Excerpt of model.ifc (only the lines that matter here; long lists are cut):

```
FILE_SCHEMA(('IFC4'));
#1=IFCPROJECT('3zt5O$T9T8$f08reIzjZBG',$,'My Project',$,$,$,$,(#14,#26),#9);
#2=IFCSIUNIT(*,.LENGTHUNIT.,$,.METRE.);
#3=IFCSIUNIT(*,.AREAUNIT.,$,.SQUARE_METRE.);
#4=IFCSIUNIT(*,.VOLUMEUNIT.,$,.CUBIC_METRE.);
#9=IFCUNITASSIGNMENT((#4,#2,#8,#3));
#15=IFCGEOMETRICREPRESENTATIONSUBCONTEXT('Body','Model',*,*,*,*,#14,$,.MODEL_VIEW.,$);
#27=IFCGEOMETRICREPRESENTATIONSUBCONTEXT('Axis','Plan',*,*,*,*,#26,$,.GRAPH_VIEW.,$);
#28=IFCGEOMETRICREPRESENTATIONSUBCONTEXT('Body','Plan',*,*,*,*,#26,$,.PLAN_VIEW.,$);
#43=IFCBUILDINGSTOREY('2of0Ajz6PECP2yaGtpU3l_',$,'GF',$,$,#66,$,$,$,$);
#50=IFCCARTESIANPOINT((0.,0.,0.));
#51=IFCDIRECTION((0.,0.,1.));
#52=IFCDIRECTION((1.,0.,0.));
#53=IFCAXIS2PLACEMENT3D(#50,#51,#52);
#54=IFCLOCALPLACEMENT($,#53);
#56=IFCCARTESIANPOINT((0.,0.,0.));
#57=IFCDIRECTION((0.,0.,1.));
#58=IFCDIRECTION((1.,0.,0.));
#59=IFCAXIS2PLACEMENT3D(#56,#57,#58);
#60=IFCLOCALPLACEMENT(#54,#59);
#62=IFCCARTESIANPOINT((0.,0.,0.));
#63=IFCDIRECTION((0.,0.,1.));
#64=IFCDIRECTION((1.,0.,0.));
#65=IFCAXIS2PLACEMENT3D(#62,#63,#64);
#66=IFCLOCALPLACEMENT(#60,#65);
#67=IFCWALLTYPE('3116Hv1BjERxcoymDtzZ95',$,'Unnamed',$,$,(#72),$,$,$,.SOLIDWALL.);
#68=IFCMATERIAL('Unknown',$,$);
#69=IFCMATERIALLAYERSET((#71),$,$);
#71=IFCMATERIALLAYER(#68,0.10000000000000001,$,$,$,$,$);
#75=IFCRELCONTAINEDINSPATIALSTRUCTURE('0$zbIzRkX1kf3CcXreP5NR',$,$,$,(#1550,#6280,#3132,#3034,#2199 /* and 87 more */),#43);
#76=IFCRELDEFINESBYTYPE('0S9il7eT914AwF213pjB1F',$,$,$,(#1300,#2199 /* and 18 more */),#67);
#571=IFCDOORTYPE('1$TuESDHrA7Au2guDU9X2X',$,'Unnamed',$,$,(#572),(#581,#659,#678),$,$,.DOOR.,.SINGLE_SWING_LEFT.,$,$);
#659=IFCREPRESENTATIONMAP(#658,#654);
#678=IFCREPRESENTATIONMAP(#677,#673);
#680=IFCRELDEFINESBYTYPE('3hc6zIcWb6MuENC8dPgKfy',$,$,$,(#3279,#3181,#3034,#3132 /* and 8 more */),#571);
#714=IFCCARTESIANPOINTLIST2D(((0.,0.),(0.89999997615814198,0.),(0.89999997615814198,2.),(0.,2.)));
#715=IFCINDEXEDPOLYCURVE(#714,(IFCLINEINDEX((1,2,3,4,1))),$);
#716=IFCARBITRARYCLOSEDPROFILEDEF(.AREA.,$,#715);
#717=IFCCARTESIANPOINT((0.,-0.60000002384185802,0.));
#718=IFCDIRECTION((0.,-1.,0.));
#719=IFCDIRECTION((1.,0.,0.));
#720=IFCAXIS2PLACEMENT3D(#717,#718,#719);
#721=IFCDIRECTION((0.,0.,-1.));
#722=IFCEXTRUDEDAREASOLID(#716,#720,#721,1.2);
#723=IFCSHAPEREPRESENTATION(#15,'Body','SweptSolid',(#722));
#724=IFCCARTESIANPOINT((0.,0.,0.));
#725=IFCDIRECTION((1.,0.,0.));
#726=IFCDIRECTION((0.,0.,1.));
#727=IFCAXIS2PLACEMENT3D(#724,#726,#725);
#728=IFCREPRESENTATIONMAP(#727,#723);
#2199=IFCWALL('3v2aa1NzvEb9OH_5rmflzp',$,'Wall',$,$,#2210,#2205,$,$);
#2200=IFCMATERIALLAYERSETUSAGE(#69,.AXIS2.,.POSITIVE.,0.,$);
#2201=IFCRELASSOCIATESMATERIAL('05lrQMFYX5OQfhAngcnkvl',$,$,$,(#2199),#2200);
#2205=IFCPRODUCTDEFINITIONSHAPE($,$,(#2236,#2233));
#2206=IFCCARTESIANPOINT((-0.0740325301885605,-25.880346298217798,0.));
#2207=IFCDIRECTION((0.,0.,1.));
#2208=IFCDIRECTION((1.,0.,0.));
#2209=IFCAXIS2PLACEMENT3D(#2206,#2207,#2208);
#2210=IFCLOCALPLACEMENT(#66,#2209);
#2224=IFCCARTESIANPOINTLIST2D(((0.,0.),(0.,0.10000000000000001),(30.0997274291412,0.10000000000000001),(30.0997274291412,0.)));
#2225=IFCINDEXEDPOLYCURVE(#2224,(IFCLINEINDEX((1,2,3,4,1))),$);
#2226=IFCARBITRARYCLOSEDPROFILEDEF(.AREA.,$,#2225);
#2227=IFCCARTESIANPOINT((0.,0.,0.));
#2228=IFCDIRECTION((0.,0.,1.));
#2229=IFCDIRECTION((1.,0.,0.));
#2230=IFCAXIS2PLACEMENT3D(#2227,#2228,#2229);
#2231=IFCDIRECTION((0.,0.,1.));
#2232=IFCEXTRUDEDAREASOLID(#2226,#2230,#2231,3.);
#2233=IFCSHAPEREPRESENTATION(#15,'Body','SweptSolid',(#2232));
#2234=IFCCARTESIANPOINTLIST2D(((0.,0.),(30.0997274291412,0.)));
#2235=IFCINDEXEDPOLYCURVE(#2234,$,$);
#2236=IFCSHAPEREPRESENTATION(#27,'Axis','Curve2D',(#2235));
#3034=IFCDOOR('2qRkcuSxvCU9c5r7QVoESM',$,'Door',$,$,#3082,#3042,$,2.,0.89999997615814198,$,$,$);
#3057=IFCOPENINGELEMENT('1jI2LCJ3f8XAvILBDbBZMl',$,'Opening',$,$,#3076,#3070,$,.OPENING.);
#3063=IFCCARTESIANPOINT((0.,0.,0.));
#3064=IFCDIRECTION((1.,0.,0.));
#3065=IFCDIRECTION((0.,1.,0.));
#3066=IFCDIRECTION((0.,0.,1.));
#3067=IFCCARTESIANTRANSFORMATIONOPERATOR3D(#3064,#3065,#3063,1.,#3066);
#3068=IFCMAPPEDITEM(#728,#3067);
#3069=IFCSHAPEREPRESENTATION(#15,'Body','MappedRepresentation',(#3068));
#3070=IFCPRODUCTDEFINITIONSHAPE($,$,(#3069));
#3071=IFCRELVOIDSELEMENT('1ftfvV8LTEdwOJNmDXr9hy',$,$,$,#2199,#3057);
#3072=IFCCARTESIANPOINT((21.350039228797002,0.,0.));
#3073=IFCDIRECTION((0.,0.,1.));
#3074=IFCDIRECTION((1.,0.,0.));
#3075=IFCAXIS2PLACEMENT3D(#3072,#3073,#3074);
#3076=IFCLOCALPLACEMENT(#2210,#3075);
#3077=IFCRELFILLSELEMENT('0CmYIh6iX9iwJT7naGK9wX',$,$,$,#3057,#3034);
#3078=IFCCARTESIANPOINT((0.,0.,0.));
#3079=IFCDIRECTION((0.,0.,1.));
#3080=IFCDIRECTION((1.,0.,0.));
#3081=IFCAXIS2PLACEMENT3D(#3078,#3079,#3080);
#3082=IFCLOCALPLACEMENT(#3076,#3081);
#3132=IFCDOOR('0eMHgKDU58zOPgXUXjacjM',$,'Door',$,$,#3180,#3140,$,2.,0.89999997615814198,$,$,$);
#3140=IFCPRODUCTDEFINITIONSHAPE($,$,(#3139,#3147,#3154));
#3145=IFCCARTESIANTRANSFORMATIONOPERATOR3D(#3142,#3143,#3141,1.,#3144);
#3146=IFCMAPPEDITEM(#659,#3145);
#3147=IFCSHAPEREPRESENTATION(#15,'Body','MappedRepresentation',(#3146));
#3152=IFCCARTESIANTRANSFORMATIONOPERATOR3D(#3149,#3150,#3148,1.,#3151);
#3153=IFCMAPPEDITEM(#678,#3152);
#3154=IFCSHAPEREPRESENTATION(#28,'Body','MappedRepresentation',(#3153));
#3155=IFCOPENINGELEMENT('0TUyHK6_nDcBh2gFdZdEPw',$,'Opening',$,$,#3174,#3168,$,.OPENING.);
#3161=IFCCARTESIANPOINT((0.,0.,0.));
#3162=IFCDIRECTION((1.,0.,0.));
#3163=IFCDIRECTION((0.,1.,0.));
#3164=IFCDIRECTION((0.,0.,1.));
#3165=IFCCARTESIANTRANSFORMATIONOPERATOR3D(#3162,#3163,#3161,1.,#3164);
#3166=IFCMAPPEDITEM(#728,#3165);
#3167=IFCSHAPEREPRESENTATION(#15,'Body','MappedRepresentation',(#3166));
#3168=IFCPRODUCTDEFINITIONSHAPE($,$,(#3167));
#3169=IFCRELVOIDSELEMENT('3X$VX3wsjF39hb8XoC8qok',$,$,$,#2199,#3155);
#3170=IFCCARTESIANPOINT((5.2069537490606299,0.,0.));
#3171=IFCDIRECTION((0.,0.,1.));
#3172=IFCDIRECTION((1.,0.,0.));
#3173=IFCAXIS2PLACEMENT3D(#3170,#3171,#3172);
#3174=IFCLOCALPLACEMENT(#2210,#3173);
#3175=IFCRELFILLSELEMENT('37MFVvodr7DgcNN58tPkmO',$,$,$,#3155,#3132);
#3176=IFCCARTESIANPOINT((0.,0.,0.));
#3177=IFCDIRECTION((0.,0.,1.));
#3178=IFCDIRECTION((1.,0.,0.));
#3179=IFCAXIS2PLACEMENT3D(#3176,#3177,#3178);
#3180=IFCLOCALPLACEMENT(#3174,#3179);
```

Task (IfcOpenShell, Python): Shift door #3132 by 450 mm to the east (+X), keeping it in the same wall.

```python
import ifcopenshell
import ifcopenshell.api.geometry
import ifcopenshell.util.placement

model = ifcopenshell.open("model.ifc")

door = model.by_id(3132)
opening = door.FillsVoids[0].RelatingOpeningElement
wall = opening.VoidsElements[0].RelatingBuildingElement

wall_matrix = ifcopenshell.util.placement.get_local_placement(wall.ObjectPlacement)
shift = wall_matrix[:3, 0] * 0.45
before = ifcopenshell.util.placement.get_local_placement(door.ObjectPlacement)[:3, 3].copy()

# The door is placed relative to its opening, so it follows when the opening moves.
matrix = ifcopenshell.util.placement.get_local_placement(opening.ObjectPlacement)
matrix[:3, 3] += shift
ifcopenshell.api.geometry.edit_object_placement(
    model, product=opening, matrix=matrix, is_si=False, should_transform_children=True
)

after = ifcopenshell.util.placement.get_local_placement(door.ObjectPlacement)[:3, 3]
print("door moved by", (after - before).round(3) + 0.0)

model.write("model-out.ifc")
```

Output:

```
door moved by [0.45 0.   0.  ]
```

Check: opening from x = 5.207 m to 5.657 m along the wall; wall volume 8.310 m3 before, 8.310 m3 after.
